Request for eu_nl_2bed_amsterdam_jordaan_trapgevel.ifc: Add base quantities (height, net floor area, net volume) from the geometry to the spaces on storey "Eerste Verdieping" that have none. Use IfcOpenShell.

First a look at what the model holds.

```python
import ifcopenshell
import ifcopenshell.util.element
import ifcopenshell.util.unit

model = ifcopenshell.open("eu_nl_2bed_amsterdam_jordaan_trapgevel.ifc")
print(model.schema)
for unit_type in ("LENGTHUNIT", "AREAUNIT", "VOLUMEUNIT"):
    print(unit_type, ifcopenshell.util.unit.calculate_unit_scale(model, unit_type))
storey = next(s for s in model.by_type("IfcBuildingStorey") if s.Name == "Eerste Verdieping")
spaces = [e for e in ifcopenshell.util.element.get_decomposition(storey) if e.is_a("IfcSpace")]
for e in sorted(spaces, key=lambda e: e.id()):
    print(e.id(), e.is_a(), e.Name, list(ifcopenshell.util.element.get_psets(e, qtos_only=True)), sep=" | ")
```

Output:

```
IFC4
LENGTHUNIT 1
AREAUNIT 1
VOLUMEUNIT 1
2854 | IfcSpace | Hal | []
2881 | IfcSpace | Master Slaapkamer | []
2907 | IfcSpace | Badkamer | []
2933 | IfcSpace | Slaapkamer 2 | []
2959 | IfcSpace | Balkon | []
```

```python
import ifcopenshell
import ifcopenshell.api.pset
import ifcopenshell.geom
import ifcopenshell.util.element
import ifcopenshell.util.shape
import ifcopenshell.util.unit

model = ifcopenshell.open("eu_nl_2bed_amsterdam_jordaan_trapgevel.ifc")
unit_scale = ifcopenshell.util.unit.calculate_unit_scale(model)
area_scale = ifcopenshell.util.unit.calculate_unit_scale(model, "AREAUNIT")
volume_scale = ifcopenshell.util.unit.calculate_unit_scale(model, "VOLUMEUNIT")
settings = ifcopenshell.geom.settings()

storey = next(s for s in model.by_type("IfcBuildingStorey") if s.Name == "Eerste Verdieping")
spaces = [e for e in ifcopenshell.util.element.get_decomposition(storey) if e.is_a("IfcSpace")]

for e in sorted(spaces, key=lambda e: e.id()):
    if ifcopenshell.util.element.get_psets(e, qtos_only=True, should_inherit=False):
        continue
    # Geometry comes back in metres, in the element's own axes.
    shape = ifcopenshell.geom.create_shape(settings, e)
    values = {
        "Height": ifcopenshell.util.shape.get_z(shape.geometry) / unit_scale,
        "NetFloorArea": ifcopenshell.util.shape.get_footprint_area(shape.geometry) / area_scale,
        "NetVolume": ifcopenshell.util.shape.get_volume(shape.geometry) / volume_scale,
    }
    qto = ifcopenshell.api.pset.add_qto(model, product=e, name="Qto_SpaceBaseQuantities")
    ifcopenshell.api.pset.edit_qto(model, qto=qto, properties=values)
    print(e.id(), {k: round(v, 3) for k, v in values.items()})

model.write("eu_nl_2bed_amsterdam_jordaan_trapgevel_v2.ifc")
```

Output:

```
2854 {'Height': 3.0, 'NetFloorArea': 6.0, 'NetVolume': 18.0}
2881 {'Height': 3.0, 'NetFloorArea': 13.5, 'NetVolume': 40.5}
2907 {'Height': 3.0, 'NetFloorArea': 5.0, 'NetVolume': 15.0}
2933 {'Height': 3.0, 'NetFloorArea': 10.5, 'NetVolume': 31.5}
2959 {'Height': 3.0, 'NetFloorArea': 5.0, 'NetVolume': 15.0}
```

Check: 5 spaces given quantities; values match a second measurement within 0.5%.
